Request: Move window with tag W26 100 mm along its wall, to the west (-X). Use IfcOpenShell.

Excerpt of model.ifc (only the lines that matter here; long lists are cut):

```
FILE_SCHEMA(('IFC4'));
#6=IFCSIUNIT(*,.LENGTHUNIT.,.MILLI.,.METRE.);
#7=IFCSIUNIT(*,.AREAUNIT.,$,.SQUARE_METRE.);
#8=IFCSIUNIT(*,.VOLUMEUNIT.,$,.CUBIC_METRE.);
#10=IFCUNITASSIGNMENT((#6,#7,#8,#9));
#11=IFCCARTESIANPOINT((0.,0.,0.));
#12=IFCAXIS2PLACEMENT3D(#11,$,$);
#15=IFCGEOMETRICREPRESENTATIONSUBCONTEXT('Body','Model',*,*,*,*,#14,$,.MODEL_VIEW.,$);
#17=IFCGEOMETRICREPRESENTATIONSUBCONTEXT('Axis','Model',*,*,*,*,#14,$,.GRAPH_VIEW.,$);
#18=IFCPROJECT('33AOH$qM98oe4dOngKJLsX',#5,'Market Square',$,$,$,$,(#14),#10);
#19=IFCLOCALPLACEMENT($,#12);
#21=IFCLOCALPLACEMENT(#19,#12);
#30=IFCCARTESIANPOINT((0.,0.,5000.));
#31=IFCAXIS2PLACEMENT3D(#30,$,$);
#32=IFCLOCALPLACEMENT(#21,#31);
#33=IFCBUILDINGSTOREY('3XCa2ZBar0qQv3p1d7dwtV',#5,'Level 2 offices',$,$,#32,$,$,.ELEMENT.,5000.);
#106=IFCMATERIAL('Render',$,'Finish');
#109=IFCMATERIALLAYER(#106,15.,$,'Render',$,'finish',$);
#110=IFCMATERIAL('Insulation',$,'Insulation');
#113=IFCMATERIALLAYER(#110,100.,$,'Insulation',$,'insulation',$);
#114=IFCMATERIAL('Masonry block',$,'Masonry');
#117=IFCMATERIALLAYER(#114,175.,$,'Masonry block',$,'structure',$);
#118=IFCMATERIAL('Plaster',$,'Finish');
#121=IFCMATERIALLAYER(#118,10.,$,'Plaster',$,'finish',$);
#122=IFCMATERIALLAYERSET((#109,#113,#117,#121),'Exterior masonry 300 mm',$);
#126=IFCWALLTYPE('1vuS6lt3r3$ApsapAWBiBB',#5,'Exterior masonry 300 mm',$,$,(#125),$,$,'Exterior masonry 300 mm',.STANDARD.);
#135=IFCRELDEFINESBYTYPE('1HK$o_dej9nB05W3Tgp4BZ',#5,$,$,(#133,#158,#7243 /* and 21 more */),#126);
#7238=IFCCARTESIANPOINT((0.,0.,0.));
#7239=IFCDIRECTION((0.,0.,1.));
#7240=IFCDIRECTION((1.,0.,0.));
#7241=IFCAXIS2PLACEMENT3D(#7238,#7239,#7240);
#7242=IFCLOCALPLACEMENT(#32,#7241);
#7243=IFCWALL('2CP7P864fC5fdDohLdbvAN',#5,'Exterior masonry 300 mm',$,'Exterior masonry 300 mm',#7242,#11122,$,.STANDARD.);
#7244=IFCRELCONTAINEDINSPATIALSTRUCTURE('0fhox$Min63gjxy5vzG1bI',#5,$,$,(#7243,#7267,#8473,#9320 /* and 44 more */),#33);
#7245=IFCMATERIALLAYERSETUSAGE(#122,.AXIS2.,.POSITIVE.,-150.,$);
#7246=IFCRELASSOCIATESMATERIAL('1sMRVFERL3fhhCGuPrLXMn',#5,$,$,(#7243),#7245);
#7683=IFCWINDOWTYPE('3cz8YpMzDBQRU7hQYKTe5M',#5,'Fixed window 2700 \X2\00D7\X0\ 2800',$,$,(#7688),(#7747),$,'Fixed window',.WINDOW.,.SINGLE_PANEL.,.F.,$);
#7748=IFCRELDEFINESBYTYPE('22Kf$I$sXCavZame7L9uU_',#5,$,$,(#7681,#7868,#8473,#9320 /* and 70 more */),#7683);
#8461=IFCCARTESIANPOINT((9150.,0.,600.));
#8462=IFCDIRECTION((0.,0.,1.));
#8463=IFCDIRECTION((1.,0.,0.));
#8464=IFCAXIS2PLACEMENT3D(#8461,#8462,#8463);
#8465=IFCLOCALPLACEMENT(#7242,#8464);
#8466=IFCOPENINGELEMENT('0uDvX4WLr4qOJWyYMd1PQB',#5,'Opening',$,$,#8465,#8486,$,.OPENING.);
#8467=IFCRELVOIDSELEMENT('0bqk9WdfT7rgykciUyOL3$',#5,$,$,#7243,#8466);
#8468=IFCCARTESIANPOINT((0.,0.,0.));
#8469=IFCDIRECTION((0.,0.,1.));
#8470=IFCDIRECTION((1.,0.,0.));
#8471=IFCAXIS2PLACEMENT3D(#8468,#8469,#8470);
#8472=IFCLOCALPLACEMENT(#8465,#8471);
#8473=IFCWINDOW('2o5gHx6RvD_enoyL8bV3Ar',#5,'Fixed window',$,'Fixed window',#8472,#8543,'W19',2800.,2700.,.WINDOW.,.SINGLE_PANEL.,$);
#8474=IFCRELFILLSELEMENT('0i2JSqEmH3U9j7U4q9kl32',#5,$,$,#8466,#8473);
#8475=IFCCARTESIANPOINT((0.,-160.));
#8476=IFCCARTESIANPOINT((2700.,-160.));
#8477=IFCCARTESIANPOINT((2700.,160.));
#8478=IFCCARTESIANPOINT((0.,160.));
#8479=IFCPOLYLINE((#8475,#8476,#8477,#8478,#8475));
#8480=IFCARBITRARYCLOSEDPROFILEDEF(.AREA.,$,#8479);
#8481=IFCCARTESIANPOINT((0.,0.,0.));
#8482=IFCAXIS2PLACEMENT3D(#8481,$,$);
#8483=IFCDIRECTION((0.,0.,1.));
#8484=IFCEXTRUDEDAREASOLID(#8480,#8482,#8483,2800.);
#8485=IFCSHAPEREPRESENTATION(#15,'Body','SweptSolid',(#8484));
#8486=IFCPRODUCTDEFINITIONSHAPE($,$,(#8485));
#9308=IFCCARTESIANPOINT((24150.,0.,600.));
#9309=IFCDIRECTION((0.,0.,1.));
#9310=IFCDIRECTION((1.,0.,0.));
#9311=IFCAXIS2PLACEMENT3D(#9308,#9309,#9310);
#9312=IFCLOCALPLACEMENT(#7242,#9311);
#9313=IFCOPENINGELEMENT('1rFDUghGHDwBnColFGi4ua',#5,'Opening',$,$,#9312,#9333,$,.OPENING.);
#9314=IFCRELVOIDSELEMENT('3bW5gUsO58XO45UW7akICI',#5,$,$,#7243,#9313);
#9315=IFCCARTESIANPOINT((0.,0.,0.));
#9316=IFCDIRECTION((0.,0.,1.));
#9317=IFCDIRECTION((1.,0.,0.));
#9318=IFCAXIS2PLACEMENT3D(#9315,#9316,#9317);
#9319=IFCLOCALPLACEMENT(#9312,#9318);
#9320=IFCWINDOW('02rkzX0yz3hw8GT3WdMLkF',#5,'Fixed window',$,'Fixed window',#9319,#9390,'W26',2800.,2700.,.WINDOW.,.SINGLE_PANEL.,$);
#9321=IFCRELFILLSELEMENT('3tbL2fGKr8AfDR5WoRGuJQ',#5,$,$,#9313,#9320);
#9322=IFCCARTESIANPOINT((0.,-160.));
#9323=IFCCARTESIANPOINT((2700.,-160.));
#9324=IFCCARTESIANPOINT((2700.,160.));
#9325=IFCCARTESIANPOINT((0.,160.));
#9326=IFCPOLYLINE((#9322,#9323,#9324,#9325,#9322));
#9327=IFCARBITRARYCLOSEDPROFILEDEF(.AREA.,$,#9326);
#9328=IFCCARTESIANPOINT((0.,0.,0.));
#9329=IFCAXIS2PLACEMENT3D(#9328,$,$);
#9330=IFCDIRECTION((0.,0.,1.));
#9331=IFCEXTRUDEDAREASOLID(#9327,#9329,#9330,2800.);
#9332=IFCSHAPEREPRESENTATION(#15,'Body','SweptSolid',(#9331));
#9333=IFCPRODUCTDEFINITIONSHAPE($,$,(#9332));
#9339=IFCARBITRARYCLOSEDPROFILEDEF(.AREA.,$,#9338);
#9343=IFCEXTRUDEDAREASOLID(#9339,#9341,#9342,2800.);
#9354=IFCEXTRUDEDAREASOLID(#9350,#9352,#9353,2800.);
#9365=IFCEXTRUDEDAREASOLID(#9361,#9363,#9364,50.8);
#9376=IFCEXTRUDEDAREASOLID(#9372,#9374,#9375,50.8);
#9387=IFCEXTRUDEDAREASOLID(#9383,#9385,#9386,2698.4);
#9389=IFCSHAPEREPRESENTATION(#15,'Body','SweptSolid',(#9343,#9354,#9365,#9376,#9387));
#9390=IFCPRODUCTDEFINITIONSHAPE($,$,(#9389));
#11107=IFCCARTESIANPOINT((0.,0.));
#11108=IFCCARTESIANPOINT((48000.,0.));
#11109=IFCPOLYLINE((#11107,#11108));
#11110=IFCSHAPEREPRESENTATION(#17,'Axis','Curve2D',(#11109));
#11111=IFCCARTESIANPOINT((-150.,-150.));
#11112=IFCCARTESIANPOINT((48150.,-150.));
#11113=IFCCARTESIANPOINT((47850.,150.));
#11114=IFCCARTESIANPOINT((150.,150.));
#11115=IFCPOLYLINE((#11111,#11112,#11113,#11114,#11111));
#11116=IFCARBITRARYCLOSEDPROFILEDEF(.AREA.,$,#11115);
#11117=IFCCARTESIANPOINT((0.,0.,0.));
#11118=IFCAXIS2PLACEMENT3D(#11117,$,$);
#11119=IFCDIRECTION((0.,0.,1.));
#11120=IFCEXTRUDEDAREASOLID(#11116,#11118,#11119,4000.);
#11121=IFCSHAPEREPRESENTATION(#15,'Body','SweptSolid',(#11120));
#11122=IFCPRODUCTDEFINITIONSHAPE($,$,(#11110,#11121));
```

```python
import ifcopenshell
import ifcopenshell.api.geometry
import ifcopenshell.util.placement

model = ifcopenshell.open("model.ifc")

window = model.by_guid("02rkzX0yz3hw8GT3WdMLkF")
opening = window.FillsVoids[0].RelatingOpeningElement
wall = opening.VoidsElements[0].RelatingBuildingElement

wall_matrix = ifcopenshell.util.placement.get_local_placement(wall.ObjectPlacement)
shift = wall_matrix[:3, 0] * -100.0
before = ifcopenshell.util.placement.get_local_placement(window.ObjectPlacement)[:3, 3].copy()

# The window is placed relative to its opening, so it follows when the opening moves.
matrix = ifcopenshell.util.placement.get_local_placement(opening.ObjectPlacement)
matrix[:3, 3] += shift
ifcopenshell.api.geometry.edit_object_placement(
    model, product=opening, matrix=matrix, is_si=False, should_transform_children=True
)

after = ifcopenshell.util.placement.get_local_placement(window.ObjectPlacement)[:3, 3]
print("window moved by", (after - before).round(3) + 0.0)

model.write("model_v2.ifc")
```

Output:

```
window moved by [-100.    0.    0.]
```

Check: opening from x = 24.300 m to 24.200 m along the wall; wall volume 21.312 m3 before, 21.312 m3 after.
